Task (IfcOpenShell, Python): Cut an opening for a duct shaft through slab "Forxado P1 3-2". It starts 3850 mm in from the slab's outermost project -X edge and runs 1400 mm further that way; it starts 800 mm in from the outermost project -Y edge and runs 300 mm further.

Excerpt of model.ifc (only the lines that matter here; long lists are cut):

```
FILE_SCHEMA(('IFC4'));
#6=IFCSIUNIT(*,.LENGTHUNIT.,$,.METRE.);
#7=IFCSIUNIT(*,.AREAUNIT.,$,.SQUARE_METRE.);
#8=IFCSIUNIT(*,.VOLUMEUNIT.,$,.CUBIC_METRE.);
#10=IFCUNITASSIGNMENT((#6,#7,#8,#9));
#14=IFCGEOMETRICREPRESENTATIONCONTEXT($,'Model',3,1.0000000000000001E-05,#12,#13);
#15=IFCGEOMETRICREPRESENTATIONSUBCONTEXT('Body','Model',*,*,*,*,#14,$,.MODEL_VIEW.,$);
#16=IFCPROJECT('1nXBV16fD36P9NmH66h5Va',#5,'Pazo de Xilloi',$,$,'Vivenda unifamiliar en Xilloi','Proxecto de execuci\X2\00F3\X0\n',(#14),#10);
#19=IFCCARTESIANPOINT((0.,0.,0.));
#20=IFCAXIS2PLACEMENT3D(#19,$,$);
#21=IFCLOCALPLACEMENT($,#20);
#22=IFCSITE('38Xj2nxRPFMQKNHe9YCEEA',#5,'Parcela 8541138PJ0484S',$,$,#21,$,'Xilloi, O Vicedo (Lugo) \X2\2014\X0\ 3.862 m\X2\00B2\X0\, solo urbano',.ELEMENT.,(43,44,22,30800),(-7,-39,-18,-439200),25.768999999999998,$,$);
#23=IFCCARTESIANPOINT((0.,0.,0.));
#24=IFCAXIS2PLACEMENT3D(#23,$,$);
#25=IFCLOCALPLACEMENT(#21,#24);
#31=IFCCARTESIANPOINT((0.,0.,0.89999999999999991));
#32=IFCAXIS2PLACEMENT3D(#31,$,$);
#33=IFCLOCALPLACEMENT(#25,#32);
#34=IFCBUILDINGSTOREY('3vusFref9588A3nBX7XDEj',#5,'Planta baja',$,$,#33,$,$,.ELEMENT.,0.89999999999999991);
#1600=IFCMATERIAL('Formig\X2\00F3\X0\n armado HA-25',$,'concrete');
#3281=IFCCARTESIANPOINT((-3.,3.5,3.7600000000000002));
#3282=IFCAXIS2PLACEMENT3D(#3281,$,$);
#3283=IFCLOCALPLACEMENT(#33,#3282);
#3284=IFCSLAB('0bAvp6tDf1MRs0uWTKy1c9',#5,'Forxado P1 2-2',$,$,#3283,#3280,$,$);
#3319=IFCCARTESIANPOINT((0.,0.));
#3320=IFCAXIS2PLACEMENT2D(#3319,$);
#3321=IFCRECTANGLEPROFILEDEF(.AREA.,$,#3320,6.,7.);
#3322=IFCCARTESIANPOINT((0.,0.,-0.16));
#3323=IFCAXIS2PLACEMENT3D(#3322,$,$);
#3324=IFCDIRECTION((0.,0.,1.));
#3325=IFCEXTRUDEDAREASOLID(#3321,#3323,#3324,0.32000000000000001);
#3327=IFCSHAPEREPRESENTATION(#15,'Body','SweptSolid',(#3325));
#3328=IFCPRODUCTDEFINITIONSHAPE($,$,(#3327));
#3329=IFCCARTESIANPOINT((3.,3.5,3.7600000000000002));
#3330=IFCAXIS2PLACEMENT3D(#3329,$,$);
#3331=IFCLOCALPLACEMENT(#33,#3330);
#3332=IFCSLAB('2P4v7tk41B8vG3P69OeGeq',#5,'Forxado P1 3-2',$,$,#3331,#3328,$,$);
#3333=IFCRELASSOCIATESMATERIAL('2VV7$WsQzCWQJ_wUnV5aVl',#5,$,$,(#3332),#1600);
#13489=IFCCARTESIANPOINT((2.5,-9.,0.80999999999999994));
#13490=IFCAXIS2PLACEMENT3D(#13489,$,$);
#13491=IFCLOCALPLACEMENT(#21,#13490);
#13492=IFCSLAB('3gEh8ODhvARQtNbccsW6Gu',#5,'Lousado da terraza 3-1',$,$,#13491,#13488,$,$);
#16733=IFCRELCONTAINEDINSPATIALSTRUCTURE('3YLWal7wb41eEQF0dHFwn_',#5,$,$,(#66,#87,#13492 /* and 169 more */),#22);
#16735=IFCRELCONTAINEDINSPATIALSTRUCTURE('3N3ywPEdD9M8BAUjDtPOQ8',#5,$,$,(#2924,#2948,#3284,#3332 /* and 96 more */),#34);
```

```python
import numpy as np
import ifcopenshell
import ifcopenshell.api.feature
import ifcopenshell.api.geometry
import ifcopenshell.api.root
import ifcopenshell.geom
import ifcopenshell.util.placement
import ifcopenshell.util.representation
import ifcopenshell.util.shape
import ifcopenshell.util.unit

model = ifcopenshell.open("model.ifc")
unit_scale = ifcopenshell.util.unit.calculate_unit_scale(model)
settings = ifcopenshell.geom.settings()


def volume(element):
    """Net volume in cubic metres, openings subtracted."""
    shape = ifcopenshell.geom.create_shape(settings, element)
    return ifcopenshell.util.shape.get_volume(shape.geometry)


slab = model.by_guid("2P4v7tk41B8vG3P69OeGeq")
before = volume(slab)

# Extent in the slab's own axes, in metres. The edges named are its -X and -Y sides.
slab_shape = ifcopenshell.geom.create_shape(settings, slab)
vertices = ifcopenshell.util.shape.get_vertices(slab_shape.geometry)
x_min, y_min, bottom = vertices.min(axis=0)
top = vertices[:, 2].max()

opening = ifcopenshell.api.root.create_entity(model, ifc_class="IfcOpeningElement", name="Duct shaft opening", predefined_type="OPENING")
context = ifcopenshell.util.representation.get_context(model, "Model", "Body", "MODEL_VIEW")
width, depth = 1.4, 0.3
outline = [(0.0, 0.0), (width, 0.0), (width, depth), (0.0, depth), (0.0, 0.0)]
# Overshoot both faces by 50 mm so the cut is clean.
shape = ifcopenshell.api.geometry.add_slab_representation(
    model, context=context, depth=top - bottom + 0.1, polyline=outline
)
ifcopenshell.api.geometry.assign_representation(model, product=opening, representation=shape)

matrix = ifcopenshell.util.placement.get_local_placement(slab.ObjectPlacement)
matrix[:, 3] = matrix @ np.append(np.array([x_min + 3.85, y_min + 0.8, bottom - 0.05]) / unit_scale, 1.0)
ifcopenshell.api.geometry.edit_object_placement(model, product=opening, matrix=matrix, is_si=False)
ifcopenshell.api.feature.add_feature(model, feature=opening, element=slab)

after = volume(slab)

print(f"slab volume {before:.3f} -> {after:.3f} m3")

model.write("model_rev.ifc")
```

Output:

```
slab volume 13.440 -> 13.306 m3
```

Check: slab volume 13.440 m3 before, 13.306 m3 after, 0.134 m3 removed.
